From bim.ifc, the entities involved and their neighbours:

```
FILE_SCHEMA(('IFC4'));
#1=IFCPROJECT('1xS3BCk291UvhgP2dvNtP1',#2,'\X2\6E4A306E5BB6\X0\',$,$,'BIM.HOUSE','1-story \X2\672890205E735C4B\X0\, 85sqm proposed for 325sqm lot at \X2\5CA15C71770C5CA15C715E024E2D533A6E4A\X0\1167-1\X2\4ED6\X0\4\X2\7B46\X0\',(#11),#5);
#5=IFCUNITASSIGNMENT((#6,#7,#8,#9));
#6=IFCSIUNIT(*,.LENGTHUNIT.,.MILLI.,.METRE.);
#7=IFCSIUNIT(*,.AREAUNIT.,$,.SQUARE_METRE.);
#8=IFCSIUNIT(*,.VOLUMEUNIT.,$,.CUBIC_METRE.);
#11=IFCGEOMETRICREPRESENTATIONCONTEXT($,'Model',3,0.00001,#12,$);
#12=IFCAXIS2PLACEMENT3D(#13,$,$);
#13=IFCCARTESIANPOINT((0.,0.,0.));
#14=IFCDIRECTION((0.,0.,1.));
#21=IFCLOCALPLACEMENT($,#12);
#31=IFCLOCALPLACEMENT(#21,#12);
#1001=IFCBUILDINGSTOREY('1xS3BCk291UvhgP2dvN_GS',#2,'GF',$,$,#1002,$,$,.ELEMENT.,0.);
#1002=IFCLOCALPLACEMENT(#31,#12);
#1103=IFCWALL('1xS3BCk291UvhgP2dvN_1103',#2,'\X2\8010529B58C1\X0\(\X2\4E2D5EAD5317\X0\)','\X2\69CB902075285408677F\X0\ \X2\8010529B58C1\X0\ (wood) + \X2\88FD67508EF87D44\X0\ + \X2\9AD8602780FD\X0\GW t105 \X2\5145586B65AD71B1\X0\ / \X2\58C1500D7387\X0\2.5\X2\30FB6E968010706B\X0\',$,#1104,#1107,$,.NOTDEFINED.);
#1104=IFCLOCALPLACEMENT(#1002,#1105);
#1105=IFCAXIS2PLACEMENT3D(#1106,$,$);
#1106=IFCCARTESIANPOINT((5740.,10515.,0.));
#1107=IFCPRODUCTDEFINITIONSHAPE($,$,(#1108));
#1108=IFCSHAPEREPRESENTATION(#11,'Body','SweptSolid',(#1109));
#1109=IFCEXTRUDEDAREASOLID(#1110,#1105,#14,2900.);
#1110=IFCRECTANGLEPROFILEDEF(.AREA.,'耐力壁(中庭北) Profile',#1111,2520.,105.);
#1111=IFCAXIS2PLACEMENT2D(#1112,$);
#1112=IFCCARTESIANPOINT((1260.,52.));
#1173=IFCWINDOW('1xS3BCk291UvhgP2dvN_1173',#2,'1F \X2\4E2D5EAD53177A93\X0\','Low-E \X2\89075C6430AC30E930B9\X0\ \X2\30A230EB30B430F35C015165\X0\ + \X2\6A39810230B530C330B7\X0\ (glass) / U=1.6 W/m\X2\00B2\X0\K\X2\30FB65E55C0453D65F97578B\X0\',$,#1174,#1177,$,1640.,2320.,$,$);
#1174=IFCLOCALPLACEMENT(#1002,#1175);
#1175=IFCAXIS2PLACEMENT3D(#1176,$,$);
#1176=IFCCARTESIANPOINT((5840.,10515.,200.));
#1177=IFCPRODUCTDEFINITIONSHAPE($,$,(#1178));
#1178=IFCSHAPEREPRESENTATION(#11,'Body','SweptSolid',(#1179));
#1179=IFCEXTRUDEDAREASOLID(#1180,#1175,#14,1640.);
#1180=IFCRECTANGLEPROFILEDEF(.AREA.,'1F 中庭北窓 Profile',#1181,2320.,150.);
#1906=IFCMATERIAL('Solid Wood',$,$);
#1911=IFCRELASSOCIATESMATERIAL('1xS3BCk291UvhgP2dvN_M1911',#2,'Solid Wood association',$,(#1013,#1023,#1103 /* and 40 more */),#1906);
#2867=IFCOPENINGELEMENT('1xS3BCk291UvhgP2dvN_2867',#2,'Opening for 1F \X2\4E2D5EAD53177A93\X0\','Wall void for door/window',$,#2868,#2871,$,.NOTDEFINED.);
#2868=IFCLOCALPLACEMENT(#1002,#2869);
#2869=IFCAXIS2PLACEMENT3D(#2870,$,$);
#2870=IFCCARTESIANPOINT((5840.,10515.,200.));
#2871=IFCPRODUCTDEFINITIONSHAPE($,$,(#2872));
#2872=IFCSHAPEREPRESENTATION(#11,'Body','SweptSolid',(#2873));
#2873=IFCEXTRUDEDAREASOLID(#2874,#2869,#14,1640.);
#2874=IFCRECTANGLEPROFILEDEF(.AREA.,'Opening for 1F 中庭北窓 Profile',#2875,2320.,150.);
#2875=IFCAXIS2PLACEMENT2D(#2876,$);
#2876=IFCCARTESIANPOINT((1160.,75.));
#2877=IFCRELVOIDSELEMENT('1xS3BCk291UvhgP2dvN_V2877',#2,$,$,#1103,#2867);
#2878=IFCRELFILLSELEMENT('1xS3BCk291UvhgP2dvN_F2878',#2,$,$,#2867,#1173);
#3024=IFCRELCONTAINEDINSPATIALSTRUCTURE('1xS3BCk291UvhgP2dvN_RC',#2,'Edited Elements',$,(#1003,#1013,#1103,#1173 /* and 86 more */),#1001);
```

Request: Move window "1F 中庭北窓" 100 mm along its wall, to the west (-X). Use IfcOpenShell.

```python
import ifcopenshell
import ifcopenshell.api.geometry
import ifcopenshell.util.placement

model = ifcopenshell.open("bim.ifc")

window = model.by_guid("1xS3BCk291UvhgP2dvN_1173")
opening = window.FillsVoids[0].RelatingOpeningElement
wall = opening.VoidsElements[0].RelatingBuildingElement

wall_matrix = ifcopenshell.util.placement.get_local_placement(wall.ObjectPlacement)
shift = wall_matrix[:3, 0] * -100.0
before = ifcopenshell.util.placement.get_local_placement(window.ObjectPlacement)[:3, 3].copy()

# The window is not placed relative to its opening, so move both.
for product in (opening, window):
    matrix = ifcopenshell.util.placement.get_local_placement(product.ObjectPlacement)
    matrix[:3, 3] += shift
    ifcopenshell.api.geometry.edit_object_placement(model, product=product, matrix=matrix, is_si=False)

after = ifcopenshell.util.placement.get_local_placement(window.ObjectPlacement)[:3, 3]
print("window moved by", (after - before).round(3) + 0.0)

model.write("bim_rev.ifc")
```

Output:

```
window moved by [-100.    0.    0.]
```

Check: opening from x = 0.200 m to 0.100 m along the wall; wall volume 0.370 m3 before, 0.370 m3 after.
